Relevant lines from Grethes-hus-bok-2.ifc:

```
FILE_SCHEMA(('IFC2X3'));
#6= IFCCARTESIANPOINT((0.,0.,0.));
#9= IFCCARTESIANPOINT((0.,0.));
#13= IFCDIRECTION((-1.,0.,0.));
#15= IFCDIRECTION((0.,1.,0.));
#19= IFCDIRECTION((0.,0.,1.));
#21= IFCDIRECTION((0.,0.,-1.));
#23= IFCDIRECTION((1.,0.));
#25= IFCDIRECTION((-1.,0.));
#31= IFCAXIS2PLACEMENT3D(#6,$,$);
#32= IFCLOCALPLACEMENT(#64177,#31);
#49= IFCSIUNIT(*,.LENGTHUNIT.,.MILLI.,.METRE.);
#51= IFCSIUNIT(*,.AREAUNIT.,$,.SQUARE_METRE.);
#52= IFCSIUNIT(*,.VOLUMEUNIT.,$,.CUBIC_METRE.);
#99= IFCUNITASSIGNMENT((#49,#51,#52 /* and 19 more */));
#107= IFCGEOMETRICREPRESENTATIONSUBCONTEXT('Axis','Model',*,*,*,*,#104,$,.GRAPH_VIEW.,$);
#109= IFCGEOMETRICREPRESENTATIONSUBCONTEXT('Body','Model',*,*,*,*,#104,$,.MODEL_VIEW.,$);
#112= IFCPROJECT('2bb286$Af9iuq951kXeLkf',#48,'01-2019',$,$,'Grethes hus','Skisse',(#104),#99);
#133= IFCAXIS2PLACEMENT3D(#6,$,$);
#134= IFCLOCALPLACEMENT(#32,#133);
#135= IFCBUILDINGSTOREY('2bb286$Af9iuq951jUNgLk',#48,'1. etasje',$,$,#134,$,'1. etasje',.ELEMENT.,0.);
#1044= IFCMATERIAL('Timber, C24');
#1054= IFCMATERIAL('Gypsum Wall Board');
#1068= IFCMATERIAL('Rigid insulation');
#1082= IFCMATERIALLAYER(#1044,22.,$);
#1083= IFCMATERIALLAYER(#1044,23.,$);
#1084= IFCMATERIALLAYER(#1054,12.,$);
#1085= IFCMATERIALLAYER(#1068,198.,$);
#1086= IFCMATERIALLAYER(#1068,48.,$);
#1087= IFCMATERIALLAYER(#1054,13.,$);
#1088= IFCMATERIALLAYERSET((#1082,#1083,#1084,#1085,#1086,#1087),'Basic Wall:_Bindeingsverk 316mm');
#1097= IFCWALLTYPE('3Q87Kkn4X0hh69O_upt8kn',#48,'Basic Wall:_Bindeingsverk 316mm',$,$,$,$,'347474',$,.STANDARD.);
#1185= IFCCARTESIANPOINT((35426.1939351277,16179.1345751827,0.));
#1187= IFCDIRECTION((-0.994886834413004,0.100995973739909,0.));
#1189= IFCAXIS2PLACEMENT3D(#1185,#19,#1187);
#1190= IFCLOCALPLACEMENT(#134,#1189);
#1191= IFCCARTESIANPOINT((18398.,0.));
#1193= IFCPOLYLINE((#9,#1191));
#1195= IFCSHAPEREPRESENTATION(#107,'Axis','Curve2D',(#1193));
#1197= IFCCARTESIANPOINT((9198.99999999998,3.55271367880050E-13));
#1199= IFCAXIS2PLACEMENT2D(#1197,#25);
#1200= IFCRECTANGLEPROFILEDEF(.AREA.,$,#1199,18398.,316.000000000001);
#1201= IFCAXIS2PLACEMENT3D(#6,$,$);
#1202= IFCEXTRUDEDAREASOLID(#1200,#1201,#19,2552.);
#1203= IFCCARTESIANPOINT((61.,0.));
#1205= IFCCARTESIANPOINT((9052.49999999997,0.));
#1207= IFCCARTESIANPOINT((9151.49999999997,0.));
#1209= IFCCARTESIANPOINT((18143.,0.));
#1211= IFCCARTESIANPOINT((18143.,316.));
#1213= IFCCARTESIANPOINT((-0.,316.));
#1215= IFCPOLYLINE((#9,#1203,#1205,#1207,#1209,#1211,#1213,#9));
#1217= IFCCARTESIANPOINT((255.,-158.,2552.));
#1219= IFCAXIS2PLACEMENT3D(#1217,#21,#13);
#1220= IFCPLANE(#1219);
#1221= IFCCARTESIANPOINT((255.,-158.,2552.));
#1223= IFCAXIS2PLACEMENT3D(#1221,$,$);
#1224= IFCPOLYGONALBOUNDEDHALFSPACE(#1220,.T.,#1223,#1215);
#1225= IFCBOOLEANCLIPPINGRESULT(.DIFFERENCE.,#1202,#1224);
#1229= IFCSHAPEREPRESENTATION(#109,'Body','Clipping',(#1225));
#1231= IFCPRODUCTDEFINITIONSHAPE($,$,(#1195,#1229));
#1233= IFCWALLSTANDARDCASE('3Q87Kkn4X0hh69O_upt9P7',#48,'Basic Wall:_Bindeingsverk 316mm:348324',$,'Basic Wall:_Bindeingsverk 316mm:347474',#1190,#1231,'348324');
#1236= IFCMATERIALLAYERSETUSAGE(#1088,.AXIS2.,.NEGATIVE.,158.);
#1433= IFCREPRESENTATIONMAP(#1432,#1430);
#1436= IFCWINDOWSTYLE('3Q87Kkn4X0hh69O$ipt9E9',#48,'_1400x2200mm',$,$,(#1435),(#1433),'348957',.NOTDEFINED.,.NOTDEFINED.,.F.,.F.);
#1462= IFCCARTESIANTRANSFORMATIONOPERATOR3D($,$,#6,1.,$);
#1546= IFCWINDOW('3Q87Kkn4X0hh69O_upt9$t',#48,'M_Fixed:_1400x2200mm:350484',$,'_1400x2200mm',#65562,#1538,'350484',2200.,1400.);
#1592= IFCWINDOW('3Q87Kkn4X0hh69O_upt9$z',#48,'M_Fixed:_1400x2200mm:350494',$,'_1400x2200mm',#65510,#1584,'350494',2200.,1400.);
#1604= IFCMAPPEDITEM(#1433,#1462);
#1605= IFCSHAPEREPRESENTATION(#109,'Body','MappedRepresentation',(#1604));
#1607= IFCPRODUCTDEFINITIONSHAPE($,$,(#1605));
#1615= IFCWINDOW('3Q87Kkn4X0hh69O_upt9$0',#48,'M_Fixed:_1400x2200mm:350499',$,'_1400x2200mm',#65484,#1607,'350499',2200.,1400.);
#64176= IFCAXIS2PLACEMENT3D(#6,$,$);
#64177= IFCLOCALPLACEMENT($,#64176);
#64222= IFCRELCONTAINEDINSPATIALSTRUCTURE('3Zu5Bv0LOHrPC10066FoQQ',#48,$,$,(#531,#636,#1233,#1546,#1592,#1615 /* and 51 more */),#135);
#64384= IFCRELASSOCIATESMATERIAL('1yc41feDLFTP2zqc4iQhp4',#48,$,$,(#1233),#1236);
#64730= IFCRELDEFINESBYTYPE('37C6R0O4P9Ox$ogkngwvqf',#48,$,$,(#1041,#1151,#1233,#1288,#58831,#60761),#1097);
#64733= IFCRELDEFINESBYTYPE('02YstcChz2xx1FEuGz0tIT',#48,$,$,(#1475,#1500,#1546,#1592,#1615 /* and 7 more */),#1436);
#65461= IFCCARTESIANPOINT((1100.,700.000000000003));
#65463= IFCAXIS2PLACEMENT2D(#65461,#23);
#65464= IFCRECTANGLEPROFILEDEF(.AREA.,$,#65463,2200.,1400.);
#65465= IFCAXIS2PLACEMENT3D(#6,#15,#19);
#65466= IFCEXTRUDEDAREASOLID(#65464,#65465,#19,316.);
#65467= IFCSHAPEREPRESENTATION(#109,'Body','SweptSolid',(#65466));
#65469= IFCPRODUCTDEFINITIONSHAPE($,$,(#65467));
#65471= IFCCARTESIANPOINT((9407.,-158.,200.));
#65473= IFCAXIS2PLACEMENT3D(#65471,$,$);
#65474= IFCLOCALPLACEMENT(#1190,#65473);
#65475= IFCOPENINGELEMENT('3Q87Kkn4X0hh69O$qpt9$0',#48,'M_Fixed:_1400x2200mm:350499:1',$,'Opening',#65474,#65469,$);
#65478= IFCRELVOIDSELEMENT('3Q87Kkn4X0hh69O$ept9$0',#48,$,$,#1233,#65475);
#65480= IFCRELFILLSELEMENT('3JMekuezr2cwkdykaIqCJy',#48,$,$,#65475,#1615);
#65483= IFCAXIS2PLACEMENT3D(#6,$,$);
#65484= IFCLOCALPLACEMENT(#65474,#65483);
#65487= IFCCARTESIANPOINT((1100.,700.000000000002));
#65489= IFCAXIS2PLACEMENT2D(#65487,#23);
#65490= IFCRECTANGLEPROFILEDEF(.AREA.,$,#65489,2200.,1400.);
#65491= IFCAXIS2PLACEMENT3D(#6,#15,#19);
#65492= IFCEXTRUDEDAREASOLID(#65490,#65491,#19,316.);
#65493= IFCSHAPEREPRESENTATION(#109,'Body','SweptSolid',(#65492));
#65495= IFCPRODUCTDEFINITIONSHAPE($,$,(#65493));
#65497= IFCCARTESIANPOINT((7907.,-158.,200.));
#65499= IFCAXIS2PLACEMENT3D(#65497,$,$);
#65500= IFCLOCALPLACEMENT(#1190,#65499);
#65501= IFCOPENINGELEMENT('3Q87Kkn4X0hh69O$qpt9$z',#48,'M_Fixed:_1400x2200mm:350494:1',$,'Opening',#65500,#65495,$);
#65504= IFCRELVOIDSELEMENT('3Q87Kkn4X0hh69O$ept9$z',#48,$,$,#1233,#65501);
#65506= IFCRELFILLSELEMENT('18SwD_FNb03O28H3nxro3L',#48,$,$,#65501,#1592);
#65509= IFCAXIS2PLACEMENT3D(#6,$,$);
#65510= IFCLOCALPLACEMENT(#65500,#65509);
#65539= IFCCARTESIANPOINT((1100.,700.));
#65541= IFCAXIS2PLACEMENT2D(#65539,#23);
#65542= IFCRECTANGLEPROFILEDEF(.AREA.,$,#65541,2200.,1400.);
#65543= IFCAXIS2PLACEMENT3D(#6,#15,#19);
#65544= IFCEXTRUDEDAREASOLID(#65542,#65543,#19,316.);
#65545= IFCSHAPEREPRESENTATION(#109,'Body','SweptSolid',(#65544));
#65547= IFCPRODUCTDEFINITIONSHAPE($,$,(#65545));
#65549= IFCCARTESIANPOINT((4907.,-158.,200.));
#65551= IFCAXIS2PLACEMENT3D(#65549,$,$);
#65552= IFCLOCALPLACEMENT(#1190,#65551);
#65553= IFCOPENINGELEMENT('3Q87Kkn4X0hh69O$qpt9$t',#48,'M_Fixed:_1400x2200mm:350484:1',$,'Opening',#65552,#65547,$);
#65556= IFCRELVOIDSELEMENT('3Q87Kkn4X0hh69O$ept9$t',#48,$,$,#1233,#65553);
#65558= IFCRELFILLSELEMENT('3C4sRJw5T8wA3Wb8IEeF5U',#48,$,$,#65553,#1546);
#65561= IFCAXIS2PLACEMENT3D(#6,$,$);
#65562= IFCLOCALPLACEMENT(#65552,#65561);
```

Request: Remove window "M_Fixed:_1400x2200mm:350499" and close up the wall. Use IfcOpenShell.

```python
import ifcopenshell
import ifcopenshell.api.feature
import ifcopenshell.api.root
import ifcopenshell.geom
import ifcopenshell.util.shape

model = ifcopenshell.open("Grethes-hus-bok-2.ifc")
settings = ifcopenshell.geom.settings()


def volume(element):
    """Net volume in cubic metres, openings subtracted."""
    shape = ifcopenshell.geom.create_shape(settings, element)
    return ifcopenshell.util.shape.get_volume(shape.geometry)


window = model.by_guid("3Q87Kkn4X0hh69O_upt9$0")
opening = window.FillsVoids[0].RelatingOpeningElement
wall = opening.VoidsElements[0].RelatingBuildingElement
before = volume(wall)

ifcopenshell.api.root.remove_product(model, product=window)
ifcopenshell.api.feature.remove_feature(model, feature=opening)

after = volume(wall)

print(f"wall volume {before:.3f} -> {after:.3f} m3")

model.write("Grethes-hus-bok-2_v2.ifc")
```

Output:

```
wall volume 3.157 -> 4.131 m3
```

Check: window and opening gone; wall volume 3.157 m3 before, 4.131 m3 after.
